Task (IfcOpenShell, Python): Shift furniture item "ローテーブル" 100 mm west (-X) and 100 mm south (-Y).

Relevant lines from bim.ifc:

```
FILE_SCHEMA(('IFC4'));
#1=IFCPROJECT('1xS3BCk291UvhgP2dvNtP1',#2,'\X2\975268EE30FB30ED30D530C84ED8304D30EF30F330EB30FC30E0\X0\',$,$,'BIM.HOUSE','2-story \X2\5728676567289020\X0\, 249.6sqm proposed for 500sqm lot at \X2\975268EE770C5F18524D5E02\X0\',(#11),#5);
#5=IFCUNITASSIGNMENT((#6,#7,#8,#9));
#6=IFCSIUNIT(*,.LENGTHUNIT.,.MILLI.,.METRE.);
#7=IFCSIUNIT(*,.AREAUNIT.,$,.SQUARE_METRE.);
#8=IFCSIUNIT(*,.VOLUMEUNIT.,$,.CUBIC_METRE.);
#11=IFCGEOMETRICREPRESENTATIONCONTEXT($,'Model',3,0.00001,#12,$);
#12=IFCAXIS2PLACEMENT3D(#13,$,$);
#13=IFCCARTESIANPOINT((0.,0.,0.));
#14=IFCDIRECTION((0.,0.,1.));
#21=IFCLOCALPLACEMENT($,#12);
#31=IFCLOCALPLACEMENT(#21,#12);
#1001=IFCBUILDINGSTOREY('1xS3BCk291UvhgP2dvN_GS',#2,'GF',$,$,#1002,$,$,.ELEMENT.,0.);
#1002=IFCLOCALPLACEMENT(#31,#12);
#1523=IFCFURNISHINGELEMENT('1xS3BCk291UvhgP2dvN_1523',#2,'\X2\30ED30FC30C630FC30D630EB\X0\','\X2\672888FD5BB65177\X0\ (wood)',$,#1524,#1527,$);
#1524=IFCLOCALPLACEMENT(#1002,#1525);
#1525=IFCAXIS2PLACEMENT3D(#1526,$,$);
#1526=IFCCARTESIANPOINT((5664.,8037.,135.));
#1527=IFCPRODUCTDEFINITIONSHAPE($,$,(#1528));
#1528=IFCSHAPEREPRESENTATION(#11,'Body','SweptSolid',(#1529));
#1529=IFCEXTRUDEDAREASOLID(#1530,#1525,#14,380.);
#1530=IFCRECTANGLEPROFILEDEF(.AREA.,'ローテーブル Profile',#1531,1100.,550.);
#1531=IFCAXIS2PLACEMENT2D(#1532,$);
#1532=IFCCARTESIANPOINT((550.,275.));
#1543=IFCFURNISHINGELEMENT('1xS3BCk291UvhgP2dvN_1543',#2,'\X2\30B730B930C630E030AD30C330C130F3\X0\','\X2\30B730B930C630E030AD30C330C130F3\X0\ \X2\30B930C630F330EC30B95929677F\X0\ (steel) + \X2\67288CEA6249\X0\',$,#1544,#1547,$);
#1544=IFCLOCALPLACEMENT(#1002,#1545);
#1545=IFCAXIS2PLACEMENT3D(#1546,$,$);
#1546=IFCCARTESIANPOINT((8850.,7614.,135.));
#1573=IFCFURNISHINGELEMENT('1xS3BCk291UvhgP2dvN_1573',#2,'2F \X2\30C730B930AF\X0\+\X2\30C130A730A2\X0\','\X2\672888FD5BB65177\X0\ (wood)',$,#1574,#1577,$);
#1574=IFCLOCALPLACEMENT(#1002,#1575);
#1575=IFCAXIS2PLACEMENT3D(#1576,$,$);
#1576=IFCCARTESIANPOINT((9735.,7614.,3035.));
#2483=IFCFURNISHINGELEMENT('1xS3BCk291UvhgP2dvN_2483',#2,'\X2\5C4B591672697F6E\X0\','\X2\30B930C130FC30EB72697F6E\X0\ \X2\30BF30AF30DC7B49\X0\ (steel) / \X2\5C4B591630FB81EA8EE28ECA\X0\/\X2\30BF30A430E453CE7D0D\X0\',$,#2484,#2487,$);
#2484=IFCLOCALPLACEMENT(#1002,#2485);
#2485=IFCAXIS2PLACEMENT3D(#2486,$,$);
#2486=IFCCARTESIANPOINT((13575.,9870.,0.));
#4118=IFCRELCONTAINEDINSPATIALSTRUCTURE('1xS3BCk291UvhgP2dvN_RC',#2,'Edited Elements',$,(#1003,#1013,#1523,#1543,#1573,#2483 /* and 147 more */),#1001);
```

```python
import ifcopenshell
import ifcopenshell.api.geometry
import ifcopenshell.util.placement
import ifcopenshell.util.unit

model = ifcopenshell.open("bim.ifc")
unit_scale = ifcopenshell.util.unit.calculate_unit_scale(model)

item = model.by_guid("1xS3BCk291UvhgP2dvN_1523")
matrix = ifcopenshell.util.placement.get_local_placement(item.ObjectPlacement)
matrix[0, 3] -= 0.1 / unit_scale
matrix[1, 3] -= 0.1 / unit_scale
ifcopenshell.api.geometry.edit_object_placement(model, product=item, matrix=matrix, is_si=False)

print(ifcopenshell.util.placement.get_local_placement(item.ObjectPlacement).round(3) + 0.0)

model.write("bim_rev.ifc")
```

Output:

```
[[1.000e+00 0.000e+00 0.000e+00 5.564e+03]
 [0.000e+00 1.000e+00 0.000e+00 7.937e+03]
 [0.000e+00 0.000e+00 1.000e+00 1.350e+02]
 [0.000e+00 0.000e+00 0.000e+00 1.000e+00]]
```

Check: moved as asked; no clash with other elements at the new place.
